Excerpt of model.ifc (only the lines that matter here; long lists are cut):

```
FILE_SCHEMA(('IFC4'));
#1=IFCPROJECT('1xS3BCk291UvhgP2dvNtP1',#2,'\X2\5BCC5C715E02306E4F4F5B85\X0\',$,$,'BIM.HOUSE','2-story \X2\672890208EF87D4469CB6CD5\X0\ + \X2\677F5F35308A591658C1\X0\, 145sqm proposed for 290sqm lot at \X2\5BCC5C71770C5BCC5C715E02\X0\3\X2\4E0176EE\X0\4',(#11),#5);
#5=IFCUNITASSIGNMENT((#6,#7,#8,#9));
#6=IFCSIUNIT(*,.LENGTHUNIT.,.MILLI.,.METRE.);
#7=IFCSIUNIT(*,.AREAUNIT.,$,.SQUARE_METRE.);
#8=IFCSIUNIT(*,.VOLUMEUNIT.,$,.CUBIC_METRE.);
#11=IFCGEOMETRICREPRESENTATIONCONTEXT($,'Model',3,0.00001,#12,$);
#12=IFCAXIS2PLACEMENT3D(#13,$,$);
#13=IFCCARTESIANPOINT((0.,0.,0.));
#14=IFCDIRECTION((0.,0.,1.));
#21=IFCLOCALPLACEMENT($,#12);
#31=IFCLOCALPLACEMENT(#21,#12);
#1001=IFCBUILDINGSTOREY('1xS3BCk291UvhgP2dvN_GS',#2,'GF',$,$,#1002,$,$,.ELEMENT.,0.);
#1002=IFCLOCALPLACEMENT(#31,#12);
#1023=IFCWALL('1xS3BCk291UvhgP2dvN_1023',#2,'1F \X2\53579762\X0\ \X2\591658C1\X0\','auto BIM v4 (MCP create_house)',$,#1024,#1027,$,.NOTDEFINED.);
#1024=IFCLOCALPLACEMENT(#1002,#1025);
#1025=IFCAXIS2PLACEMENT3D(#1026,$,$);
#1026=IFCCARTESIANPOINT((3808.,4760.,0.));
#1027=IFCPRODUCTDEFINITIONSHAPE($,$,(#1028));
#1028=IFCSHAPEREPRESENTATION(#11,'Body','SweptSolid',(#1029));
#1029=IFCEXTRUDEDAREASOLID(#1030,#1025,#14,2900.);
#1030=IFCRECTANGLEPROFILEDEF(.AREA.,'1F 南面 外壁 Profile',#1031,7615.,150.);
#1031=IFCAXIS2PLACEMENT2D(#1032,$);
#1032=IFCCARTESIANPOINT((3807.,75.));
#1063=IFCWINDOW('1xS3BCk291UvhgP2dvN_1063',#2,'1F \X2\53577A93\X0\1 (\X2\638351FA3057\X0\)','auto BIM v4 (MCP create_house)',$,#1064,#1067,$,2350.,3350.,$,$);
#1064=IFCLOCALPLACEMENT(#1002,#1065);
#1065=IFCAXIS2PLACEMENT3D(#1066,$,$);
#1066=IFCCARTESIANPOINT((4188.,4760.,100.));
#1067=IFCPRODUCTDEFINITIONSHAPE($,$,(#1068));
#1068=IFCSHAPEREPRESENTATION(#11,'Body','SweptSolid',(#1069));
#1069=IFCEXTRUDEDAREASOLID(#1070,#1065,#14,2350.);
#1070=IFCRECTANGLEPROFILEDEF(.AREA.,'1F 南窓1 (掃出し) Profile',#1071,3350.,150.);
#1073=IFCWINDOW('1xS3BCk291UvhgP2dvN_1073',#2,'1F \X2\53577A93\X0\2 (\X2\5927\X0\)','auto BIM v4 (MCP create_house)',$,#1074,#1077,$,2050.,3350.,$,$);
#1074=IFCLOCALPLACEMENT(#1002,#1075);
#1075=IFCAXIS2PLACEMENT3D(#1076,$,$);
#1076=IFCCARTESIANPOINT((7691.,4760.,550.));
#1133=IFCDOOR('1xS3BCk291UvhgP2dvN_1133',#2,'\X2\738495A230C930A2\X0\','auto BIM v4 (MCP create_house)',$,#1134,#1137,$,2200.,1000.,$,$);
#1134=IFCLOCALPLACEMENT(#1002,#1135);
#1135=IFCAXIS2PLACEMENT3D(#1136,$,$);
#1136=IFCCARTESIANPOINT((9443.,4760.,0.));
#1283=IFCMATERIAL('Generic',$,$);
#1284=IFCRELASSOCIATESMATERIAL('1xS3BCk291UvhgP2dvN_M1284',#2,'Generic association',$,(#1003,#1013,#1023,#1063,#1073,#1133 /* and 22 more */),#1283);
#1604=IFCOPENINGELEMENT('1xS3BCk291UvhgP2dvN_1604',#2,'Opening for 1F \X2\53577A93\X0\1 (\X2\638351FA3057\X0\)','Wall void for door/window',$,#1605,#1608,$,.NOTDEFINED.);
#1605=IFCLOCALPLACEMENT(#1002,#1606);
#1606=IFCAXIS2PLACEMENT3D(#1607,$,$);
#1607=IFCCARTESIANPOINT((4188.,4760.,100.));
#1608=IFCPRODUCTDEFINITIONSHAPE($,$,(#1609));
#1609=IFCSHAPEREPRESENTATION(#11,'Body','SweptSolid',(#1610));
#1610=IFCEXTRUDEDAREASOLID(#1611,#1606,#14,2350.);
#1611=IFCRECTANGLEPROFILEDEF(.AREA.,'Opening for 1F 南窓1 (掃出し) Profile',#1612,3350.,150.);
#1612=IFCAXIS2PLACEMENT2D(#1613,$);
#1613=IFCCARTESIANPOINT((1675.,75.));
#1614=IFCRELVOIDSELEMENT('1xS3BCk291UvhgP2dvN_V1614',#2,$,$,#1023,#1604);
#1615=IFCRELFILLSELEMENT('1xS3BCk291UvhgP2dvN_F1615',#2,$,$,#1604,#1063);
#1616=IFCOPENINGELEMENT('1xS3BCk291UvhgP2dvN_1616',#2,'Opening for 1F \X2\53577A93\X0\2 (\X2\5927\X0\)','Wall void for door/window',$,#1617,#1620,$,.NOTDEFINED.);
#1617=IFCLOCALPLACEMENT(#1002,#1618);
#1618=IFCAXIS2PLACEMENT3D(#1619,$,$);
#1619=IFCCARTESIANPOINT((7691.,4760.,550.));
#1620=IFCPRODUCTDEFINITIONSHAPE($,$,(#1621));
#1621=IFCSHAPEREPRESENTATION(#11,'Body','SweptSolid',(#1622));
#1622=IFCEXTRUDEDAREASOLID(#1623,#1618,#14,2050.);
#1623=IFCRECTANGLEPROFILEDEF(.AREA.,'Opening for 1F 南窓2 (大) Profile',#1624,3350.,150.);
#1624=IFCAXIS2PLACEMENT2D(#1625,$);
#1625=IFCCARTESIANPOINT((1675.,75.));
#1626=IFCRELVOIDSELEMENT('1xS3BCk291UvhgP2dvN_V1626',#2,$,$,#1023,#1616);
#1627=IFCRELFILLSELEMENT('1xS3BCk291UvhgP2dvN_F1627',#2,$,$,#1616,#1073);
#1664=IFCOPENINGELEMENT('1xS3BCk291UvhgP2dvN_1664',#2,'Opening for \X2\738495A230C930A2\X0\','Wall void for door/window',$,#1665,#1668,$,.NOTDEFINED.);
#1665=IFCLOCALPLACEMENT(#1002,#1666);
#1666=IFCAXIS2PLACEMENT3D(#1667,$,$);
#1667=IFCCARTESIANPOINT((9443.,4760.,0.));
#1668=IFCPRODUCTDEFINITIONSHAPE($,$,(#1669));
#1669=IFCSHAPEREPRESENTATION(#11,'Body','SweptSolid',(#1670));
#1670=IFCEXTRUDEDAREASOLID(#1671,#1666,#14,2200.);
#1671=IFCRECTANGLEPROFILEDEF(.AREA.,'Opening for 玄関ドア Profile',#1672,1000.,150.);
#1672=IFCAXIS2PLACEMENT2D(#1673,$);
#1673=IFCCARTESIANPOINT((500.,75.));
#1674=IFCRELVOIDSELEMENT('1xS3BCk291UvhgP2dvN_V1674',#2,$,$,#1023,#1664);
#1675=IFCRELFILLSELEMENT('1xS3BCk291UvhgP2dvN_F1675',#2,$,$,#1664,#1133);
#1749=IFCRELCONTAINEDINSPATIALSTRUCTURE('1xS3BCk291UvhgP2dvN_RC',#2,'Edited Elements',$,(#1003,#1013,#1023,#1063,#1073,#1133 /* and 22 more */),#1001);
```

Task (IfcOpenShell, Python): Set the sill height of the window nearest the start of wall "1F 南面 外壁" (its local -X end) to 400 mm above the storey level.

```python
import numpy as np
import ifcopenshell
import ifcopenshell.api.geometry
import ifcopenshell.geom
import ifcopenshell.util.element
import ifcopenshell.util.placement
import ifcopenshell.util.shape
import ifcopenshell.util.unit

model = ifcopenshell.open("model.ifc")
unit_scale = ifcopenshell.util.unit.calculate_unit_scale(model)

window = model.by_id(1063)
opening = window.FillsVoids[0].RelatingOpeningElement
storey = ifcopenshell.util.element.get_container(window, ifc_class="IfcBuildingStorey")
level = ifcopenshell.util.placement.get_local_placement(storey.ObjectPlacement)[2, 3]

# The opening's origin need not be at the sill, so measure its lowest point.
shape = ifcopenshell.geom.create_shape(ifcopenshell.geom.settings(), opening)
bottom = ifcopenshell.util.shape.get_shape_bottom_elevation(shape, shape.geometry) / unit_scale
dz = level + 0.4 / unit_scale - bottom

shift = np.array([0.0, 0.0, dz])
# The window is not placed relative to its opening, so move both.
for product in (opening, window):
    matrix = ifcopenshell.util.placement.get_local_placement(product.ObjectPlacement)
    matrix[:3, 3] += shift
    ifcopenshell.api.geometry.edit_object_placement(model, product=product, matrix=matrix, is_si=False)

print(f"moved by {dz * unit_scale:+.3f} m")

model.write("model_updated.ifc")
```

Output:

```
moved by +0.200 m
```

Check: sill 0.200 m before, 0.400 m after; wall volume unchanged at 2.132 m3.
